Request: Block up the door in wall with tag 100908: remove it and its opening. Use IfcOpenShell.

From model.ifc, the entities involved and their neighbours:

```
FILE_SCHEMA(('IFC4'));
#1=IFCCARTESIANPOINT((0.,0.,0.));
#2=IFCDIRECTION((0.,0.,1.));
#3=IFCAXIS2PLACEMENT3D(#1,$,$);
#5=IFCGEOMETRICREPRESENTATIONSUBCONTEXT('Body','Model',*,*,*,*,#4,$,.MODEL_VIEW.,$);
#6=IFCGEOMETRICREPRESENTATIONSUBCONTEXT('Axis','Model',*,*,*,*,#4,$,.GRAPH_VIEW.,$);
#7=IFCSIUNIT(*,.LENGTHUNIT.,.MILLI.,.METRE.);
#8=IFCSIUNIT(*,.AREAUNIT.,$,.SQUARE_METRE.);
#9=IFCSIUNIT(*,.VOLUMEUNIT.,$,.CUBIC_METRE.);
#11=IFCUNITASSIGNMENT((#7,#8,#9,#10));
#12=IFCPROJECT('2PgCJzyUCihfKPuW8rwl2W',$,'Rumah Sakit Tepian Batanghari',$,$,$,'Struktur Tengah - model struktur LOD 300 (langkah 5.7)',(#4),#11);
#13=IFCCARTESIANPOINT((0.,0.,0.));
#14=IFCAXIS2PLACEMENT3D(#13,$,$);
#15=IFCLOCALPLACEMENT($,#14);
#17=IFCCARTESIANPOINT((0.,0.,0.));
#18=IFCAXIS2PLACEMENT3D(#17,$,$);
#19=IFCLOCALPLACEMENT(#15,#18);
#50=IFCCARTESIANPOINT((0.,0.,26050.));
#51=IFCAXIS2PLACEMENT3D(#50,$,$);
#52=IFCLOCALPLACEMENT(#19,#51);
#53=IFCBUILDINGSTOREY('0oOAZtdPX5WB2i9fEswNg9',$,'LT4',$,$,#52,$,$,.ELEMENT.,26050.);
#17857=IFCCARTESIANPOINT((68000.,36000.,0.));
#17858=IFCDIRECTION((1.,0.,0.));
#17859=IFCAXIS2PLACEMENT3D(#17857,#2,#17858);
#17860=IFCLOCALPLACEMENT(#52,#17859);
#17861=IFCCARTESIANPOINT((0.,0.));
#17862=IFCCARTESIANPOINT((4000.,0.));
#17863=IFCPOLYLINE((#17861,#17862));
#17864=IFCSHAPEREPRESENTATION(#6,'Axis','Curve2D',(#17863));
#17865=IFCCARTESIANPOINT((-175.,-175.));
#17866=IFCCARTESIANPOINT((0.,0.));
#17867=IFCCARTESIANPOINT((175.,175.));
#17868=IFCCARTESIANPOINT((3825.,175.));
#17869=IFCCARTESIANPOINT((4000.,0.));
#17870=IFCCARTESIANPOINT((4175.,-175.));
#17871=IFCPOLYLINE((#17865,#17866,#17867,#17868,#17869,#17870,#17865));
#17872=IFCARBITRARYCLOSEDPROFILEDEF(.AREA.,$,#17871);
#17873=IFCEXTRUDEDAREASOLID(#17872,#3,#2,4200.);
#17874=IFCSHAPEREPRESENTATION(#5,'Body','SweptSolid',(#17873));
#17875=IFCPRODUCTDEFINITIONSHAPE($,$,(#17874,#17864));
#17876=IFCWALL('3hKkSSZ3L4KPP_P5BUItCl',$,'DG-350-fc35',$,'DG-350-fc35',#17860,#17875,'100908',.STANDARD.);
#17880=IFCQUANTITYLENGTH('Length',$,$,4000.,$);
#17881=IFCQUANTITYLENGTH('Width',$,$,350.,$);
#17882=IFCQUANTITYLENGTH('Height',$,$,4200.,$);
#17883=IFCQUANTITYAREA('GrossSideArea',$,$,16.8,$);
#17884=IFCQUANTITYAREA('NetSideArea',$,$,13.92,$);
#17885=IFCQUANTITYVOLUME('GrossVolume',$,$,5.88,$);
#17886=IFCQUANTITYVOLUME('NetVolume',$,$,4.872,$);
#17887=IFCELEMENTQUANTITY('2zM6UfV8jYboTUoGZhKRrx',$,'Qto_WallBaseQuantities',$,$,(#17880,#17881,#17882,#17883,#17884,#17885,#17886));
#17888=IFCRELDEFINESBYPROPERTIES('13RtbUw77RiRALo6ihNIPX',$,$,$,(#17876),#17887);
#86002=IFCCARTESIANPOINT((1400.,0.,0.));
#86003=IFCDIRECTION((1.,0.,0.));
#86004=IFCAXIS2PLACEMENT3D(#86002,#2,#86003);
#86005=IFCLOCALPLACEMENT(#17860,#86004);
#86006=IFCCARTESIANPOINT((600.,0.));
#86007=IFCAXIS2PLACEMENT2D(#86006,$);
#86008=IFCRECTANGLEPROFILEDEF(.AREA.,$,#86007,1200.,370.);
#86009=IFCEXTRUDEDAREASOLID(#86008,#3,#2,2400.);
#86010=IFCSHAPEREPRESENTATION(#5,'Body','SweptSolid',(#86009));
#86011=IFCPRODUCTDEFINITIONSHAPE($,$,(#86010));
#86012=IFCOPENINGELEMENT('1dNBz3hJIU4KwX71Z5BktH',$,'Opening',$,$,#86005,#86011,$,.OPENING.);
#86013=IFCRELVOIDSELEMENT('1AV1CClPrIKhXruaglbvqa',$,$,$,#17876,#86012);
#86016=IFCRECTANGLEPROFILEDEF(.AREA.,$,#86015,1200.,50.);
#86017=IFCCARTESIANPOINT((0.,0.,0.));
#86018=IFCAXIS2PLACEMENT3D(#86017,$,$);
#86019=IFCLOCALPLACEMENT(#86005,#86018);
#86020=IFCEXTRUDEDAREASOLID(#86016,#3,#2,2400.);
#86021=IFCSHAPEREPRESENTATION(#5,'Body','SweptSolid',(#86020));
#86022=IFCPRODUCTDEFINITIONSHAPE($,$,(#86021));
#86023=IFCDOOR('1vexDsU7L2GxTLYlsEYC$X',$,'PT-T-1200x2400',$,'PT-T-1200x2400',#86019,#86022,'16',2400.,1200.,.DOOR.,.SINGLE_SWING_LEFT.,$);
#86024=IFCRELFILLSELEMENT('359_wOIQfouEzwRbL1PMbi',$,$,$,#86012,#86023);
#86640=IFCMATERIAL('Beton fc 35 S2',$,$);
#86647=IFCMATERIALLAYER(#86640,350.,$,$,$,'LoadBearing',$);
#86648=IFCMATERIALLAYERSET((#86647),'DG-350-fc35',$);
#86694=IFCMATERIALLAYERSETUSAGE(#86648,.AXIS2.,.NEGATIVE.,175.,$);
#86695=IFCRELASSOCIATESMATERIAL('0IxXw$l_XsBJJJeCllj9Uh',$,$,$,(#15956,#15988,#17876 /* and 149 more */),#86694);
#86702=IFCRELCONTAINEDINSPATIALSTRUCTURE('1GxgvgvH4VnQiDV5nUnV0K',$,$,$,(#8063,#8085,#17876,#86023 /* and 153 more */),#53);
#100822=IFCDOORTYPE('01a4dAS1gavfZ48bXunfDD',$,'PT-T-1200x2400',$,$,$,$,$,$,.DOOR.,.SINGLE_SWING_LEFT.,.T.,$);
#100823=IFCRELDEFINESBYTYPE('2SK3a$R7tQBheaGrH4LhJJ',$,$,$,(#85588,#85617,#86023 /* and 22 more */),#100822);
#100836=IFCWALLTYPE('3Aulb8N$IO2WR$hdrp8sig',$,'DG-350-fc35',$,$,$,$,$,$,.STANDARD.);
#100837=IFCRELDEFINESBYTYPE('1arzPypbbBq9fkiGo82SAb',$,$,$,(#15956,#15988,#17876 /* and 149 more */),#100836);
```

```python
import ifcopenshell
import ifcopenshell.api.feature
import ifcopenshell.api.pset
import ifcopenshell.api.root
import ifcopenshell.geom
import ifcopenshell.util.element
import ifcopenshell.util.shape
import ifcopenshell.util.unit

model = ifcopenshell.open("model.ifc")
area_scale = ifcopenshell.util.unit.calculate_unit_scale(model, "AREAUNIT")
volume_scale = ifcopenshell.util.unit.calculate_unit_scale(model, "VOLUMEUNIT")
settings = ifcopenshell.geom.settings()


def volume(element):
    """Net volume in cubic metres, openings subtracted."""
    shape = ifcopenshell.geom.create_shape(settings, element)
    return ifcopenshell.util.shape.get_volume(shape.geometry)


door = model.by_guid("1vexDsU7L2GxTLYlsEYC$X")
opening = door.FillsVoids[0].RelatingOpeningElement
wall = opening.VoidsElements[0].RelatingBuildingElement
before = volume(wall)

ifcopenshell.api.root.remove_product(model, product=door)
ifcopenshell.api.feature.remove_feature(model, feature=opening)

after = volume(wall)
thickness = 0.35  # wall thickness in metres

# Update the wall's stored quantities.
qto = model.by_id(ifcopenshell.util.element.get_pset(wall, "Qto_WallBaseQuantities", should_inherit=False)["id"])
ifcopenshell.api.pset.edit_qto(model, qto=qto, properties={
    "NetSideArea": after / thickness / area_scale,
    "NetVolume": after / volume_scale,
})

print(f"wall volume {before:.3f} -> {after:.3f} m3")

model.write("model-out.ifc")
```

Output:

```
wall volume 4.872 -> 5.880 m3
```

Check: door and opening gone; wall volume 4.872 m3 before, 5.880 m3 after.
